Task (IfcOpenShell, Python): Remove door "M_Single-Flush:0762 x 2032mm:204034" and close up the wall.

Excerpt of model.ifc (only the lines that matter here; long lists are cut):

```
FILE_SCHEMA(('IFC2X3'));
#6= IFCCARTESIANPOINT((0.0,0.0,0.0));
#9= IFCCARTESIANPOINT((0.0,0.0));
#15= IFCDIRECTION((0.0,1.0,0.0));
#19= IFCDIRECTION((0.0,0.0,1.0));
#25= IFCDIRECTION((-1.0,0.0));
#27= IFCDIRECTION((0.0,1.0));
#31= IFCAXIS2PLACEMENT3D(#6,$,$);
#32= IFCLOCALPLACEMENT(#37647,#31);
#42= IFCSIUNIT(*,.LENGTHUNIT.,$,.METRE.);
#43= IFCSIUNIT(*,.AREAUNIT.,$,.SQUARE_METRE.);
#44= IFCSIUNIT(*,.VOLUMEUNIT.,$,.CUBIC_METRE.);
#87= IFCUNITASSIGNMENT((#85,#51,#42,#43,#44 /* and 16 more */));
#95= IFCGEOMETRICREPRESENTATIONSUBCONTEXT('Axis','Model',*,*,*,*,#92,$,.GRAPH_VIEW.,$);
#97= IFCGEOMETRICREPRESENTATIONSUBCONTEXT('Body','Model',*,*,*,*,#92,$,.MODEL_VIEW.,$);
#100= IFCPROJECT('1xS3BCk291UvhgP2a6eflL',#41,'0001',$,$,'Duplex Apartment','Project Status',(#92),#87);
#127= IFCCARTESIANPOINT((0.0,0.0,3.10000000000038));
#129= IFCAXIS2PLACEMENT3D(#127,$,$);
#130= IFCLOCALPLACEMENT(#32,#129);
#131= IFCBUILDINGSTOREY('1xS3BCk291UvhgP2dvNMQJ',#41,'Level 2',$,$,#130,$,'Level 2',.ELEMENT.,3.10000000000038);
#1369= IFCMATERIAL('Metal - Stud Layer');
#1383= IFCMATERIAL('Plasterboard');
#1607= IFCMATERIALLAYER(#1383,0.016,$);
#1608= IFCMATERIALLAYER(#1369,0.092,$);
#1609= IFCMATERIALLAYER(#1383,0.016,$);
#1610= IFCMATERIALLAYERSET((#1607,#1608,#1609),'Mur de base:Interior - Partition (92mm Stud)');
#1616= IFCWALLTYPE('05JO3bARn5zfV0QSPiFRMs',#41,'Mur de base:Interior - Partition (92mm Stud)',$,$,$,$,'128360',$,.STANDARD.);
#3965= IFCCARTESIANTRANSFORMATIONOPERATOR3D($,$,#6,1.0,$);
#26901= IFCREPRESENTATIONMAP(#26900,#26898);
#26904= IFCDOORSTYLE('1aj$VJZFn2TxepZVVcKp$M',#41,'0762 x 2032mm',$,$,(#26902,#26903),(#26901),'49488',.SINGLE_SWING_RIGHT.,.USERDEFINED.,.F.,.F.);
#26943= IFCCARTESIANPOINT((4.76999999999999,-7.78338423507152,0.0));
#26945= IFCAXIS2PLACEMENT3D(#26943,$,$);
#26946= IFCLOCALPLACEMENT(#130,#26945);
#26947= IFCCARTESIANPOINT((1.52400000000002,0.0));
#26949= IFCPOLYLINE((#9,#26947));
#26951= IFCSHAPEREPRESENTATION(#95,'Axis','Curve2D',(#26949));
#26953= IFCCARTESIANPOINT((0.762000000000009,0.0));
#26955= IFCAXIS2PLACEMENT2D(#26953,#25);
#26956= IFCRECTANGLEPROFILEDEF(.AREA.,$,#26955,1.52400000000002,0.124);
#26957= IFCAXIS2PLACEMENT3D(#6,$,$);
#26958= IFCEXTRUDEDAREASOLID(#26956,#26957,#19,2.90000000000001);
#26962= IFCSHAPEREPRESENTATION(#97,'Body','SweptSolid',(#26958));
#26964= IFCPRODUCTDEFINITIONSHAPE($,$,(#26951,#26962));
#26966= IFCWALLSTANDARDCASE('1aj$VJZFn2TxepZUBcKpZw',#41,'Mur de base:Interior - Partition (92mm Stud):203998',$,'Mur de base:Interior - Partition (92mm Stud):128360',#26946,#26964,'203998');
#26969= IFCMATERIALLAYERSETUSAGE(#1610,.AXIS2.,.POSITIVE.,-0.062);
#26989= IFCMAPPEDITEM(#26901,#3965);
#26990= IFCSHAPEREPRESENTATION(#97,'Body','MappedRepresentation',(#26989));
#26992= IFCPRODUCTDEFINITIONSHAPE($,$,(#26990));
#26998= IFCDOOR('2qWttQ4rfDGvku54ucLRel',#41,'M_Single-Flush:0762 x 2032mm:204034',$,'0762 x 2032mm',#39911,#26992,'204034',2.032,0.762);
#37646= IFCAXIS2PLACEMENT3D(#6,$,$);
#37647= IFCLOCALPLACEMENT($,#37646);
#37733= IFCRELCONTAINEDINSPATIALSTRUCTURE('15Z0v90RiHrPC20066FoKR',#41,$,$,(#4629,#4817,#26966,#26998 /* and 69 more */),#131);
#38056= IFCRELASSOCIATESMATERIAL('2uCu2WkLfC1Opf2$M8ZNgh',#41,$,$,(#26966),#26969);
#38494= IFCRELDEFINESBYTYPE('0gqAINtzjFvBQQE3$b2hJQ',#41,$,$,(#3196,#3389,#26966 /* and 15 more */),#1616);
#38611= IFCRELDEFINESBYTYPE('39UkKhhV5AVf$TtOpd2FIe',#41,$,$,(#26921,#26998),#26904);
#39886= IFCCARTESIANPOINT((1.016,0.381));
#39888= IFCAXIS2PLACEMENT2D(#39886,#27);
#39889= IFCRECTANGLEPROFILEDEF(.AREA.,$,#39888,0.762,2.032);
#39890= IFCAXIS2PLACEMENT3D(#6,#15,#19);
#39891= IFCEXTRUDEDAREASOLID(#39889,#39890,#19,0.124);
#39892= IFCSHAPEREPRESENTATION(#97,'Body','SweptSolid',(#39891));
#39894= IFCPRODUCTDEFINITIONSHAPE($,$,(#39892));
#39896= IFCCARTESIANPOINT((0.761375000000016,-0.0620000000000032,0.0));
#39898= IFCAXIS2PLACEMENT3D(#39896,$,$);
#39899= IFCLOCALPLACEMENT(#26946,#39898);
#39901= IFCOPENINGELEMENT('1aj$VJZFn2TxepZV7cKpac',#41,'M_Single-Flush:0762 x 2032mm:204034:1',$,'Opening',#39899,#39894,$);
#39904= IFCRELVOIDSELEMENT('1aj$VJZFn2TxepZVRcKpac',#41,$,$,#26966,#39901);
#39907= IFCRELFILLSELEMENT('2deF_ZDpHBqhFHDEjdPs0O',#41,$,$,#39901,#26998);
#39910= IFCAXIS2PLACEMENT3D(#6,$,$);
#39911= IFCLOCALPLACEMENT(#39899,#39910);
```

```python
import ifcopenshell
import ifcopenshell.api.feature
import ifcopenshell.api.root
import ifcopenshell.geom
import ifcopenshell.util.shape

model = ifcopenshell.open("model.ifc")
settings = ifcopenshell.geom.settings()


def volume(element):
    """Net volume in cubic metres, openings subtracted."""
    shape = ifcopenshell.geom.create_shape(settings, element)
    return ifcopenshell.util.shape.get_volume(shape.geometry)


door = model.by_guid("2qWttQ4rfDGvku54ucLRel")
opening = door.FillsVoids[0].RelatingOpeningElement
wall = opening.VoidsElements[0].RelatingBuildingElement
before = volume(wall)

ifcopenshell.api.root.remove_product(model, product=door)
ifcopenshell.api.feature.remove_feature(model, feature=opening)

after = volume(wall)

print(f"wall volume {before:.3f} -> {after:.3f} m3")

model.write("model_updated.ifc")
```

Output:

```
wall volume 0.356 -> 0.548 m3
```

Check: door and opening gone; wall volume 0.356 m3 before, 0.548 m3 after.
